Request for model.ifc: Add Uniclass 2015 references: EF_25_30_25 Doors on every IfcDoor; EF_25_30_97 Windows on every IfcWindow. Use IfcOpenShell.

First a look at what the model holds.

```python
import ifcopenshell

model = ifcopenshell.open("model.ifc")
print(model.schema)
print("classifications:", [c.Name for c in model.by_type("IfcClassification")])
for ifc_class in ("IfcDoor", "IfcRoof", "IfcStair", "IfcWall", "IfcWindow"):
    print(ifc_class, len(model.by_type(ifc_class)))
```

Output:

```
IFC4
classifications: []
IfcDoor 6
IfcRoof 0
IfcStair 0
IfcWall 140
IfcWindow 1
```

```python
import ifcopenshell
import ifcopenshell.api.classification

model = ifcopenshell.open("model.ifc")

system = ifcopenshell.api.classification.add_classification(model, classification="Uniclass 2015")

codes = {
    "IfcDoor": ("EF_25_30_25", "Doors"),
    "IfcWindow": ("EF_25_30_97", "Windows"),
}
for ifc_class, (code, name) in codes.items():
    products = model.by_type(ifc_class)
    ifcopenshell.api.classification.add_reference(
        model, products=products, classification=system, identification=code, name=name
    )
    print(code, len(products))

model.write("model_updated.ifc")
```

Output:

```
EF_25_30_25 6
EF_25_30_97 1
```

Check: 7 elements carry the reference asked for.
